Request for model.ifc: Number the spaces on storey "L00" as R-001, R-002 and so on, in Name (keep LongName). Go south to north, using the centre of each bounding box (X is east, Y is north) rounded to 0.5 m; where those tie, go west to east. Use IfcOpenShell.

First a look at what the model holds.

```python
import ifcopenshell
import ifcopenshell.util.element
import ifcopenshell.util.placement

model = ifcopenshell.open("model.ifc")
print(model.schema)
storey = next(s for s in model.by_type("IfcBuildingStorey") if s.Name == "L00")
spaces = [e for e in ifcopenshell.util.element.get_decomposition(storey) if e.is_a("IfcSpace")]
for e in sorted(spaces, key=lambda e: e.id()):
    origin = ifcopenshell.util.placement.get_local_placement(e.ObjectPlacement)[:3, 3]
    print(e.id(), e.Name, e.LongName, origin.round(2) + 0.0, sep=" | ")
```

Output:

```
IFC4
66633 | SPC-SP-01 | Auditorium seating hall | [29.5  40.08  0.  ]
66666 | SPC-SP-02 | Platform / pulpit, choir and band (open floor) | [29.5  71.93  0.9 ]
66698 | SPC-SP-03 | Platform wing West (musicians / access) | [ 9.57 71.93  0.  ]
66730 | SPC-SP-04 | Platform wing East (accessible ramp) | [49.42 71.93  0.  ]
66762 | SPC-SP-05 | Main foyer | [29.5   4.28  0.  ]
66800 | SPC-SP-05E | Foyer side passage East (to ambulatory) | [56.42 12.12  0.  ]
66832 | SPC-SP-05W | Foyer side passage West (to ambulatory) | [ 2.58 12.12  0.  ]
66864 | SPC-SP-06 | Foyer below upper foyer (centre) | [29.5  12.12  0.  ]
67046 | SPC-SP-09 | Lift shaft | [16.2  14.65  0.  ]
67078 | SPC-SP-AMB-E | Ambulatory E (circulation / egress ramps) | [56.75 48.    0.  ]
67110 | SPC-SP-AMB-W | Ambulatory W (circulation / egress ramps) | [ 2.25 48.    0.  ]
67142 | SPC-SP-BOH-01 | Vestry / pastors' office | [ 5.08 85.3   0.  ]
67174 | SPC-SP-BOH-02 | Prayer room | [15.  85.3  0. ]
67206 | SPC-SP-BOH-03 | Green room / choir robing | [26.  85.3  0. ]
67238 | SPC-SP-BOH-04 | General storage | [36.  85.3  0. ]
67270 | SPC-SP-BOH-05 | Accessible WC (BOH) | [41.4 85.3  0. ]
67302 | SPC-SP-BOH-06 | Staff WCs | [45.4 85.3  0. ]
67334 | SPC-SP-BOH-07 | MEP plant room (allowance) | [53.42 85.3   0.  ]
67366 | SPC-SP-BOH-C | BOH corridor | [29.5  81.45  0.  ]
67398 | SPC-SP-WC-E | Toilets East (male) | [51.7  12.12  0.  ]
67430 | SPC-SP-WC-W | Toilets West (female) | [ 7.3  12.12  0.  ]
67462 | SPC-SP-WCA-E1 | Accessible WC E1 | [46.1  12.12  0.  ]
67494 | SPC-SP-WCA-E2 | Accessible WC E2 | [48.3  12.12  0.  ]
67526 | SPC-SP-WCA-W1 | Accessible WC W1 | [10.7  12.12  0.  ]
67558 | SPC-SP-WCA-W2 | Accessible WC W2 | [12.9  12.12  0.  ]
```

```python
import ifcopenshell
import ifcopenshell.geom
import ifcopenshell.util.element
import ifcopenshell.util.shape

model = ifcopenshell.open("model.ifc")
settings = ifcopenshell.geom.settings()
settings.set("use-world-coords", True)


def centre(element):
    shape = ifcopenshell.geom.create_shape(settings, element)
    return ifcopenshell.util.shape.get_bbox_centroid(shape.geometry)


storey = next(s for s in model.by_type("IfcBuildingStorey") if s.Name == "L00")
spaces = [e for e in ifcopenshell.util.element.get_decomposition(storey) if e.is_a("IfcSpace")]

# Insertion points can sit at a corner or the storey origin, so sort by the geometry (in metres).
centres = {e: centre(e) for e in spaces}
spaces.sort(key=lambda e: (round(centres[e][1] / 0.5), centres[e][0]))

for i, e in enumerate(spaces, start=1):
    number = f"R-0{i:02d}"
    e.Name = number
    print(e.id(), number)

model.write("model_v2.ifc")
```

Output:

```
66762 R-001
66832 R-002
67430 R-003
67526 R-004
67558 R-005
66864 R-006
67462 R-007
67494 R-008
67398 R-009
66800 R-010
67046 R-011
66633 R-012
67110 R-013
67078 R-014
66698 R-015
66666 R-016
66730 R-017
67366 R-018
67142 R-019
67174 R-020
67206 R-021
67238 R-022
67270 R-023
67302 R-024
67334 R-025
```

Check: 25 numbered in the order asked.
